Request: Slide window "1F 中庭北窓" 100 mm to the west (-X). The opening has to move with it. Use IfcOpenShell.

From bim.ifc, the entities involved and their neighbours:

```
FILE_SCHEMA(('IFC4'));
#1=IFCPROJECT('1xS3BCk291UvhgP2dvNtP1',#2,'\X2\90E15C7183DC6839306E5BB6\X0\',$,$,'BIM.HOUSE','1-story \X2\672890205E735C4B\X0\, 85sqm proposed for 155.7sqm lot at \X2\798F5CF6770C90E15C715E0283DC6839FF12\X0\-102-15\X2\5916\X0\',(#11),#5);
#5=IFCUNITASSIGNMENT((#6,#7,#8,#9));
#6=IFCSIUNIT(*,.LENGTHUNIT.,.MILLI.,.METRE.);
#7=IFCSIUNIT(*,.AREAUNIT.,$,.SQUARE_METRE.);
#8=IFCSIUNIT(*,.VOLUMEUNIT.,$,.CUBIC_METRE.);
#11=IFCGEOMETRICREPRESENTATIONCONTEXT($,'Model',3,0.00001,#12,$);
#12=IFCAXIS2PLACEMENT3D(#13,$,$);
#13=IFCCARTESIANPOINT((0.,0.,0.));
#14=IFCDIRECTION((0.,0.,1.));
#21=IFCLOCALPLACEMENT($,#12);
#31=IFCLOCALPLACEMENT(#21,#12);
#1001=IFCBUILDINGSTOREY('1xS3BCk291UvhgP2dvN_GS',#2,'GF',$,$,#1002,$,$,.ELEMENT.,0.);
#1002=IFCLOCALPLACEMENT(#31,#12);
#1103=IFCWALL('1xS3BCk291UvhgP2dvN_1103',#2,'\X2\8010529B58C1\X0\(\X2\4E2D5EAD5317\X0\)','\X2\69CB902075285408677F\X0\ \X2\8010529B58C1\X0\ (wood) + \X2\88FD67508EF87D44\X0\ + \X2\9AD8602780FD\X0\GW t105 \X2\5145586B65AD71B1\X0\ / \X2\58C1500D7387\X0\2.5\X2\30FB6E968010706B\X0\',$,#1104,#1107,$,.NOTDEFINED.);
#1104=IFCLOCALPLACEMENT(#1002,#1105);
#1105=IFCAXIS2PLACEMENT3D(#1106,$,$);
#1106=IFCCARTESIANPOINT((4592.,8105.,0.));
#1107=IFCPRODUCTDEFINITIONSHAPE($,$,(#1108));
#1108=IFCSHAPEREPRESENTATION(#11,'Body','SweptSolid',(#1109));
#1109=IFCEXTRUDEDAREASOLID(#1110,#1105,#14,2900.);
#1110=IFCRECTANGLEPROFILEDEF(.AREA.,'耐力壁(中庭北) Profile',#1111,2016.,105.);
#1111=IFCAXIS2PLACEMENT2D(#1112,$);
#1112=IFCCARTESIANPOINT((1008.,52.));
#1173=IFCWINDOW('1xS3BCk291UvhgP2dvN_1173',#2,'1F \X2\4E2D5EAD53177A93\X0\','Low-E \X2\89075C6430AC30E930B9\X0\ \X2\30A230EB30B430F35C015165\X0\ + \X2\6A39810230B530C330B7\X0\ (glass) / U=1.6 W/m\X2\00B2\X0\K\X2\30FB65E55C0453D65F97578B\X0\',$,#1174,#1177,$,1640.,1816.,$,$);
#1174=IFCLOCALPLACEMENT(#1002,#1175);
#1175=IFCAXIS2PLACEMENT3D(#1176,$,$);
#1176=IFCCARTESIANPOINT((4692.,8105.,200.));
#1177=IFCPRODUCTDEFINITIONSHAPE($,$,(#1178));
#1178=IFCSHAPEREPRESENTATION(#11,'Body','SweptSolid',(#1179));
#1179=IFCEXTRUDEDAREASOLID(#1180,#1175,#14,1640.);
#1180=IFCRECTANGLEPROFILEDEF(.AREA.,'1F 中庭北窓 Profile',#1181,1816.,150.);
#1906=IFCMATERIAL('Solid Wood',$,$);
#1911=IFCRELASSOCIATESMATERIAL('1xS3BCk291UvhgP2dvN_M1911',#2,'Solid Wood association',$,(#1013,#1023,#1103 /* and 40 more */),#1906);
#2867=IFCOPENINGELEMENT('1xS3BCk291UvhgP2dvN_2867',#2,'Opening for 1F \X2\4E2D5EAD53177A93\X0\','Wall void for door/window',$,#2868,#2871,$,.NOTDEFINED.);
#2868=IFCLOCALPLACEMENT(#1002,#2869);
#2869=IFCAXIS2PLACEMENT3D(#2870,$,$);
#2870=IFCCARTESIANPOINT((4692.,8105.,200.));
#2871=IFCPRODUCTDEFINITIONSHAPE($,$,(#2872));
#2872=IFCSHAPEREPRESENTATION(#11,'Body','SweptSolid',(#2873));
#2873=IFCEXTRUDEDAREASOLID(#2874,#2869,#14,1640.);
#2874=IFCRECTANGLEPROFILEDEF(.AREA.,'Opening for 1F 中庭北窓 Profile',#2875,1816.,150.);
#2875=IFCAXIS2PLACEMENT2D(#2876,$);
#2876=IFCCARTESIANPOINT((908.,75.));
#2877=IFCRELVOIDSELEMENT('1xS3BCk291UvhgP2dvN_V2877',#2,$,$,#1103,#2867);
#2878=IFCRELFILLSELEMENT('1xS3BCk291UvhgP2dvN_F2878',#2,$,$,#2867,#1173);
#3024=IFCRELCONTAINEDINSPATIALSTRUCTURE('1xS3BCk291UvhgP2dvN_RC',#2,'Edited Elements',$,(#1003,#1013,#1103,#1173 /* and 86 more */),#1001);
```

```python
import ifcopenshell
import ifcopenshell.api.geometry
import ifcopenshell.util.placement

model = ifcopenshell.open("bim.ifc")

window = model.by_guid("1xS3BCk291UvhgP2dvN_1173")
opening = window.FillsVoids[0].RelatingOpeningElement
wall = opening.VoidsElements[0].RelatingBuildingElement

wall_matrix = ifcopenshell.util.placement.get_local_placement(wall.ObjectPlacement)
shift = wall_matrix[:3, 0] * -100.0
before = ifcopenshell.util.placement.get_local_placement(window.ObjectPlacement)[:3, 3].copy()

# The window is not placed relative to its opening, so move both.
for product in (opening, window):
    matrix = ifcopenshell.util.placement.get_local_placement(product.ObjectPlacement)
    matrix[:3, 3] += shift
    ifcopenshell.api.geometry.edit_object_placement(model, product=product, matrix=matrix, is_si=False)

after = ifcopenshell.util.placement.get_local_placement(window.ObjectPlacement)[:3, 3]
print("window moved by", (after - before).round(3) + 0.0)

model.write("bim_v2.ifc")
```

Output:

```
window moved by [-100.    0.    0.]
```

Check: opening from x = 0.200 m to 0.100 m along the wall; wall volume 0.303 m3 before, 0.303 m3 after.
